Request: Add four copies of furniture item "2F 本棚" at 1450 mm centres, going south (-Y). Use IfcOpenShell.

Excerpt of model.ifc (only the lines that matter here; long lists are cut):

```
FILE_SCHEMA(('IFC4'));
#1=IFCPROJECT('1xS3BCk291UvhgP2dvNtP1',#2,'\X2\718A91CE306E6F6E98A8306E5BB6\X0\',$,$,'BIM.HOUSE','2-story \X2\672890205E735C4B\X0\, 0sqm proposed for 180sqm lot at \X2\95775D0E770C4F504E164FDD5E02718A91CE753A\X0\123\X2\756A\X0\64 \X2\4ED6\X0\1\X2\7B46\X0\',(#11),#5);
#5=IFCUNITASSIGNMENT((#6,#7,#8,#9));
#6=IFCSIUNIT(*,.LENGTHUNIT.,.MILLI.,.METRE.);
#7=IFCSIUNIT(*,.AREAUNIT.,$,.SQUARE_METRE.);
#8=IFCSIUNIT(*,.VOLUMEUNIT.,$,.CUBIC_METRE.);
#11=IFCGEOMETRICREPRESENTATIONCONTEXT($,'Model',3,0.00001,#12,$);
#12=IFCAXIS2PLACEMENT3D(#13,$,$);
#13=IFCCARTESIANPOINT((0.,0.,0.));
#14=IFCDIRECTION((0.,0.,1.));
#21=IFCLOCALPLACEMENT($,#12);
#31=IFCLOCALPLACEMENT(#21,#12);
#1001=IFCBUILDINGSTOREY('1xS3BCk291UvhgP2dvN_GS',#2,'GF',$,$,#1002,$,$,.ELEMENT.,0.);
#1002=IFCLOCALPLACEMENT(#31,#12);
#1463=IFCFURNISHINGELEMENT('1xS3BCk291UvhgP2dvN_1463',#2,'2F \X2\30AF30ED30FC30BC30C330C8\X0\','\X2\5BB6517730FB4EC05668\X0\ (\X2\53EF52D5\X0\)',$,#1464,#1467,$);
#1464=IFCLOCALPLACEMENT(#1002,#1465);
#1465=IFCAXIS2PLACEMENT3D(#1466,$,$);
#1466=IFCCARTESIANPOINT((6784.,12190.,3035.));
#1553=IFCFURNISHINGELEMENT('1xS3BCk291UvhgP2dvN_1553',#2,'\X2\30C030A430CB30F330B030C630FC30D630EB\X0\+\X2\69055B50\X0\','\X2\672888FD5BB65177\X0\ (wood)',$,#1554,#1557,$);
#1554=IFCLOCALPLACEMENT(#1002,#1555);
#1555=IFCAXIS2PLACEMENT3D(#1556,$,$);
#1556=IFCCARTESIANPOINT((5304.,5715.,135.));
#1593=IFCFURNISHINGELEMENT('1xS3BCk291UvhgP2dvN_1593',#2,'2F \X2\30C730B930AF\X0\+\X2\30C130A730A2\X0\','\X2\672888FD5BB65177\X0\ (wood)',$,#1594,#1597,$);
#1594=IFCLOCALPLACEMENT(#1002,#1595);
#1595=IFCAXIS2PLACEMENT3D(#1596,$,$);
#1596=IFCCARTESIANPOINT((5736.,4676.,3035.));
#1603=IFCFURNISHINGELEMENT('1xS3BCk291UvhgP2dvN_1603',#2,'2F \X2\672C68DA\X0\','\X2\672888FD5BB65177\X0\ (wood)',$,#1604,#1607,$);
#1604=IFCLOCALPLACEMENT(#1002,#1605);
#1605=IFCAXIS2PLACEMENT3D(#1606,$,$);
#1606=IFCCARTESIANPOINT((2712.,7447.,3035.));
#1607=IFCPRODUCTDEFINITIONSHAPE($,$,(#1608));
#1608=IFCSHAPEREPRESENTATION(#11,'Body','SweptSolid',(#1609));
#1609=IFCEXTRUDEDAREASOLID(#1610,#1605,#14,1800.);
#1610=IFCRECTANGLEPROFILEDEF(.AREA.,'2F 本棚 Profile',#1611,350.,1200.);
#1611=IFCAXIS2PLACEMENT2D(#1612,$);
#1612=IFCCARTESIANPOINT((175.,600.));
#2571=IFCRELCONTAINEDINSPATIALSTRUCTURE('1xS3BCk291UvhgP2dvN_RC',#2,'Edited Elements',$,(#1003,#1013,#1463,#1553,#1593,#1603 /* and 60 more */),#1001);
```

```python
import numpy as np
import ifcopenshell
import ifcopenshell.api.geometry
import ifcopenshell.api.root
import ifcopenshell.util.element
import ifcopenshell.util.placement

model = ifcopenshell.open("model.ifc")


def reuse_history(source, copy):
    """copy_class also copies each property set's owner history, people and application; keep the originals."""
    for rel in copy.IsDefinedBy:
        if rel.is_a("IfcRelDefinesByProperties") and (history := rel.RelatingPropertyDefinition.OwnerHistory):
            rel.RelatingPropertyDefinition.OwnerHistory = source.OwnerHistory
            ifcopenshell.util.element.remove_deep2(model, history)


source = model.by_guid("1xS3BCk291UvhgP2dvN_1603")
base = ifcopenshell.util.placement.get_local_placement(source.ObjectPlacement)
step = np.array([0.0, -1.0, 0.0]) * 1450.0

for i in range(1, 5):
    copy = ifcopenshell.api.root.copy_class(model, product=source)
    copy.Representation = ifcopenshell.util.element.copy_deep(
        model, source.Representation, exclude=["IfcGeometricRepresentationContext", "IfcRepresentationMap"]
    )
    reuse_history(source, copy)
    matrix = base.copy()
    matrix[:3, 3] += i * step
    print("added at", matrix[:3, 3].round(3) + 0.0)
    ifcopenshell.api.geometry.edit_object_placement(model, product=copy, matrix=matrix, is_si=False)

model.write("model_v2.ifc")
```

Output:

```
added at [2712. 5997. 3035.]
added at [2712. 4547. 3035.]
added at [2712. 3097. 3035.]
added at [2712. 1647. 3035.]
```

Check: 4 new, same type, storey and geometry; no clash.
